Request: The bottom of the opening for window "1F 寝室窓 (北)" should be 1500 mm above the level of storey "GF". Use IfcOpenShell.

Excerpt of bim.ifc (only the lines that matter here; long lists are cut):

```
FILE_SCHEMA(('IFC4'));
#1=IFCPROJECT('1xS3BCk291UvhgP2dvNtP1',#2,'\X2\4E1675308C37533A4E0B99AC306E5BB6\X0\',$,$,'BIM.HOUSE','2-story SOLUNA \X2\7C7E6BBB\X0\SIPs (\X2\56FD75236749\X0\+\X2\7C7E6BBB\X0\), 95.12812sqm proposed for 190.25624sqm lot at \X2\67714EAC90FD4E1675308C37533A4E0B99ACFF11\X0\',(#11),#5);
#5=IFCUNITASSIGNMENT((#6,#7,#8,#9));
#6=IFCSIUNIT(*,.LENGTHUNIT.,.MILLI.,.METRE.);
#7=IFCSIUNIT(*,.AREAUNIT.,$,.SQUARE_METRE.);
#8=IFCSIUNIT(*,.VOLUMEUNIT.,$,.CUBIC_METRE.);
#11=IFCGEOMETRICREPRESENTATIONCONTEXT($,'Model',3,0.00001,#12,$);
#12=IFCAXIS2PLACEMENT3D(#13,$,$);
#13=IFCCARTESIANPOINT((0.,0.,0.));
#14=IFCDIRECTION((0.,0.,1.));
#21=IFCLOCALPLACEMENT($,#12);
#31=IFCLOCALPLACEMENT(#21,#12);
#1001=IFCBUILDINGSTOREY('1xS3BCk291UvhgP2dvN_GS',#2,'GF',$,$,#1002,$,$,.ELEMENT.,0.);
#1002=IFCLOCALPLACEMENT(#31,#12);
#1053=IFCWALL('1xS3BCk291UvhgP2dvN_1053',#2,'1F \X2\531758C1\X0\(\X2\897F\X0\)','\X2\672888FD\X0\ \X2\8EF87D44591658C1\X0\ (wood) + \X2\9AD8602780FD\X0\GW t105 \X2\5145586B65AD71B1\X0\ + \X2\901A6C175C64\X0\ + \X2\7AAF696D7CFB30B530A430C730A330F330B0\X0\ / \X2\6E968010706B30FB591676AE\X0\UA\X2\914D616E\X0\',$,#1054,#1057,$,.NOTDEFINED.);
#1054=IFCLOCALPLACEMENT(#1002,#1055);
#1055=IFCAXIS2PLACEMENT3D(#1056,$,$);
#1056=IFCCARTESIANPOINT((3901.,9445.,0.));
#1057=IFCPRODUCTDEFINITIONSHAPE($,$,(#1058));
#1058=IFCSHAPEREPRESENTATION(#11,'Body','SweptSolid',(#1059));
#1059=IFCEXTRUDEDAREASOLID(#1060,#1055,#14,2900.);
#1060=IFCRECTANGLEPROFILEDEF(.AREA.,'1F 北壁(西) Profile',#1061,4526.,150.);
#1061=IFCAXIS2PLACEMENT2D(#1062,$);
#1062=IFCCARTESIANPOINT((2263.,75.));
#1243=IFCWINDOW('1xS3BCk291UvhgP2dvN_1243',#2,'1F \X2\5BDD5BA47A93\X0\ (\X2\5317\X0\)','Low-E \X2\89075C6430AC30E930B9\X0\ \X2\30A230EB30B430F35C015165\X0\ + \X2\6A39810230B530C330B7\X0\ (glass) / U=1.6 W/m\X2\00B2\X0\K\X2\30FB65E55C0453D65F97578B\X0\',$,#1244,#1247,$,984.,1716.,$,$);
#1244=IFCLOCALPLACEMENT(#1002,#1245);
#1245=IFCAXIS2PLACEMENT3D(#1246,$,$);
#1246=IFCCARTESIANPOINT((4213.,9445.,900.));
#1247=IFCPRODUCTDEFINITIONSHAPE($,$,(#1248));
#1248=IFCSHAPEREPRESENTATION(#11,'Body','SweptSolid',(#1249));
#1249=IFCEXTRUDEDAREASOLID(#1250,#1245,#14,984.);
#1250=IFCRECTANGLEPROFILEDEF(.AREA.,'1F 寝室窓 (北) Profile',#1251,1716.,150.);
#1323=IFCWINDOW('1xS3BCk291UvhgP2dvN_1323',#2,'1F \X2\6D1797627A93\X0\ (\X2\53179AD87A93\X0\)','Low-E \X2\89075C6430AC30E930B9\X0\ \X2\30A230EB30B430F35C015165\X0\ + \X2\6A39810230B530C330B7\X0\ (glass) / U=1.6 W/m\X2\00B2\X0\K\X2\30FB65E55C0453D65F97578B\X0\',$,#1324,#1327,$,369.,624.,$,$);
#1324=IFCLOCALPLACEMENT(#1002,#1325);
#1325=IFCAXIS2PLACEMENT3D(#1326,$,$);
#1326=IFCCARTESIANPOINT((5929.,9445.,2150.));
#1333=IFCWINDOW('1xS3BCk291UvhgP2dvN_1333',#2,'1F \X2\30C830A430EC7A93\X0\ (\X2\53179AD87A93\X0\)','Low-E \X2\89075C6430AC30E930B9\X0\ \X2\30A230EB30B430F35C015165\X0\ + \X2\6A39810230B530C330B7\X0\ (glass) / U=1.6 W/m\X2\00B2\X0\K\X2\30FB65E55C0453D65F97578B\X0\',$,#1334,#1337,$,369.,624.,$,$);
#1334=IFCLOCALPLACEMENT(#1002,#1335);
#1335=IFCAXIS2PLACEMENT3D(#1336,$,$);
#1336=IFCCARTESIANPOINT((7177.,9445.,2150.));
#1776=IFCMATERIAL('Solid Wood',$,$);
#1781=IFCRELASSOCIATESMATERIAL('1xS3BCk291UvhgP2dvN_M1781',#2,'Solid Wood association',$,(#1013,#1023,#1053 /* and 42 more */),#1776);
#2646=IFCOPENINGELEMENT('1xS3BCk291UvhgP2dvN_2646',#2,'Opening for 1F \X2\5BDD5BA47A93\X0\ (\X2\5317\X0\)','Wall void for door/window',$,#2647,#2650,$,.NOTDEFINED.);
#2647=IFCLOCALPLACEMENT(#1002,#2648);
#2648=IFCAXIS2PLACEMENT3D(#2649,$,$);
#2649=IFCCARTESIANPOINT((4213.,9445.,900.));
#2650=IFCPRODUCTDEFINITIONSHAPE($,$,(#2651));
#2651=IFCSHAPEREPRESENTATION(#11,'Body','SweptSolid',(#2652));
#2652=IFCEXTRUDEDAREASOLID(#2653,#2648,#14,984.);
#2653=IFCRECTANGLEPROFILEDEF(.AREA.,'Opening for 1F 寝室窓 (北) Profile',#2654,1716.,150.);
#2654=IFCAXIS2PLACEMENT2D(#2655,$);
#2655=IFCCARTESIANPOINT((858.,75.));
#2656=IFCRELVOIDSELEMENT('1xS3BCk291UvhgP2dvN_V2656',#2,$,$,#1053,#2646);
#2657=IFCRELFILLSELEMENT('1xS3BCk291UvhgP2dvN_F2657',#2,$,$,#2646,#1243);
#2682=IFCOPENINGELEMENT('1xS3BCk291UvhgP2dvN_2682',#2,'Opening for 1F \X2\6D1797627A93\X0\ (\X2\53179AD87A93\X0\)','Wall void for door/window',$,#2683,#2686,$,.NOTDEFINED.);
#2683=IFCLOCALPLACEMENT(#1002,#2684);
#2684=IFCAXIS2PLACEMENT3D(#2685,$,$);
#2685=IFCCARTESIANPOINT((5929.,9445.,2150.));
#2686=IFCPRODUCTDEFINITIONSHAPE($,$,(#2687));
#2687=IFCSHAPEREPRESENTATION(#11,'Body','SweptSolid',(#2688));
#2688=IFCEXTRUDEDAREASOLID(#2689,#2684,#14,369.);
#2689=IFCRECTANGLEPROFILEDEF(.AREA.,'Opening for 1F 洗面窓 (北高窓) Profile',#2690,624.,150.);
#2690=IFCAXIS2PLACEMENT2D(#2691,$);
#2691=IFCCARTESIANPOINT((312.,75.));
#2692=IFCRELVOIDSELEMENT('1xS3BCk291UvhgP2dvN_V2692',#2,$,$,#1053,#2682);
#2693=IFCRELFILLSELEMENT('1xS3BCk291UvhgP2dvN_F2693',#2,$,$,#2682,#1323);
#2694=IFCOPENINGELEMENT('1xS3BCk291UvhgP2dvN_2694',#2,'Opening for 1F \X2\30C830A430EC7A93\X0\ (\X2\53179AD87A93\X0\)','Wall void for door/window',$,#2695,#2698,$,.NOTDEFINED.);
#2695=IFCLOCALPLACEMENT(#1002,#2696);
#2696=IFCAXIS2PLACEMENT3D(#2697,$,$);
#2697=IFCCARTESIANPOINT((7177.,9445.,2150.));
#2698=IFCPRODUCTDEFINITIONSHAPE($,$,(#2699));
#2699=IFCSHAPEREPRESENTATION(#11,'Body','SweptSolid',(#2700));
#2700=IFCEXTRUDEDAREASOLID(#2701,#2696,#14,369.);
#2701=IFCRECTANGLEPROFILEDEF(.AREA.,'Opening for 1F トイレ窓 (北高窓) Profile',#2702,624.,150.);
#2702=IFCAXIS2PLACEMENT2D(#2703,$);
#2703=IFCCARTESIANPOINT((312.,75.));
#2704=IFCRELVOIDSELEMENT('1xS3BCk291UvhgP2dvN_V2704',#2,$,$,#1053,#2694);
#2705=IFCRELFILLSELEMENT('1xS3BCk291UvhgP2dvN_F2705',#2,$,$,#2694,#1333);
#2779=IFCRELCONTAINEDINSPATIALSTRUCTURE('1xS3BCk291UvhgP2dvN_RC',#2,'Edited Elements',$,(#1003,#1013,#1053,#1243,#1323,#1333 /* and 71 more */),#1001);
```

```python
import numpy as np
import ifcopenshell
import ifcopenshell.api.geometry
import ifcopenshell.geom
import ifcopenshell.util.element
import ifcopenshell.util.placement
import ifcopenshell.util.shape
import ifcopenshell.util.unit

model = ifcopenshell.open("bim.ifc")
unit_scale = ifcopenshell.util.unit.calculate_unit_scale(model)

window = model.by_id(1243)
opening = window.FillsVoids[0].RelatingOpeningElement
storey = ifcopenshell.util.element.get_container(window, ifc_class="IfcBuildingStorey")
level = ifcopenshell.util.placement.get_local_placement(storey.ObjectPlacement)[2, 3]

# The opening's origin need not be at the sill, so measure its lowest point.
shape = ifcopenshell.geom.create_shape(ifcopenshell.geom.settings(), opening)
bottom = ifcopenshell.util.shape.get_shape_bottom_elevation(shape, shape.geometry) / unit_scale
dz = level + 1.5 / unit_scale - bottom

shift = np.array([0.0, 0.0, dz])
# The window is not placed relative to its opening, so move both.
for product in (opening, window):
    matrix = ifcopenshell.util.placement.get_local_placement(product.ObjectPlacement)
    matrix[:3, 3] += shift
    ifcopenshell.api.geometry.edit_object_placement(model, product=product, matrix=matrix, is_si=False)

print(f"moved by {dz * unit_scale:+.3f} m")

model.write("bim_updated.ifc")
```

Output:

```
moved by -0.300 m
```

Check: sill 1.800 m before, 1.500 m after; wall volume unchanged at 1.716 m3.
